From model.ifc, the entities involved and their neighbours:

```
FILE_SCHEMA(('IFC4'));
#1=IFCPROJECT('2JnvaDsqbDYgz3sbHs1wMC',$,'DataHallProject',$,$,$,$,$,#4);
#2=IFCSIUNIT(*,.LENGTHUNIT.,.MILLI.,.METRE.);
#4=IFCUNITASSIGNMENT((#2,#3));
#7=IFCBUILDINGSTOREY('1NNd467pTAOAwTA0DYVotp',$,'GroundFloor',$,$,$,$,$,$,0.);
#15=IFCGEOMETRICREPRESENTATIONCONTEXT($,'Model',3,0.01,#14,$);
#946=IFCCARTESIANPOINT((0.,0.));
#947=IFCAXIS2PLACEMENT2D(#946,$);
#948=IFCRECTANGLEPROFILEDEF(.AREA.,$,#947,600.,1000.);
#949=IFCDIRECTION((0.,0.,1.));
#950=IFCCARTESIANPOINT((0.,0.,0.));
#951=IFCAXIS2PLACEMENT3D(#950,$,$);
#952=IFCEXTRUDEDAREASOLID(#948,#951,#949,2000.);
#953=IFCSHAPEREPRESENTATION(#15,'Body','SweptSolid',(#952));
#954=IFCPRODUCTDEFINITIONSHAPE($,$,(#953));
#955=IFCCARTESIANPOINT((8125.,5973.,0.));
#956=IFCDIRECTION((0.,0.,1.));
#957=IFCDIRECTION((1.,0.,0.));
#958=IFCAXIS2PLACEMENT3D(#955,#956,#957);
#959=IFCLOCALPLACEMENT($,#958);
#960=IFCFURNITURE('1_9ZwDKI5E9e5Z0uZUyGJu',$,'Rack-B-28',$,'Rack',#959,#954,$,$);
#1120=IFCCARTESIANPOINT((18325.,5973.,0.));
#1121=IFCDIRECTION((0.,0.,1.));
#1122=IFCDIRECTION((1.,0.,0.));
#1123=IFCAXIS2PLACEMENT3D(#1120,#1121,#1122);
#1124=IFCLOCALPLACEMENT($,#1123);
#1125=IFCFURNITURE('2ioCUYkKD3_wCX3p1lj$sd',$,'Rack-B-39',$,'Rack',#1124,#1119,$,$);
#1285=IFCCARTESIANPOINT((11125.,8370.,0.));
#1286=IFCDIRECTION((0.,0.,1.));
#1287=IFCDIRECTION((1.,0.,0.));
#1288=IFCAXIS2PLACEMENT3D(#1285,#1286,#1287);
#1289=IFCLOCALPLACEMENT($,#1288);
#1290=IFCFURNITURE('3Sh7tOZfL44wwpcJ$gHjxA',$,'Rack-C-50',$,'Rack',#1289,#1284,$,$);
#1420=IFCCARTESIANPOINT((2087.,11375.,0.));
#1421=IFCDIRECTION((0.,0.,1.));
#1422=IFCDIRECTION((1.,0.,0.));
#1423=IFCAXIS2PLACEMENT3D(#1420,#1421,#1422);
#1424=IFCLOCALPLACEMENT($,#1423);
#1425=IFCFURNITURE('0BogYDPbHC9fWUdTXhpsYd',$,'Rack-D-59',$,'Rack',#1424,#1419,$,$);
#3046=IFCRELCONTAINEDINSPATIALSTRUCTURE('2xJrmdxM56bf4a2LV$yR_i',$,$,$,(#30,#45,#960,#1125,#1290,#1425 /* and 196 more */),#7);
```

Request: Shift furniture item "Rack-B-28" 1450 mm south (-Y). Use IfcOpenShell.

```python
import ifcopenshell
import ifcopenshell.api.geometry
import ifcopenshell.util.placement

model = ifcopenshell.open("model.ifc")

item = model.by_id(960)
matrix = ifcopenshell.util.placement.get_local_placement(item.ObjectPlacement)
matrix[1, 3] -= 1450.0
ifcopenshell.api.geometry.edit_object_placement(model, product=item, matrix=matrix, is_si=False)

print(ifcopenshell.util.placement.get_local_placement(item.ObjectPlacement).round(3) + 0.0)

model.write("model_updated.ifc")
```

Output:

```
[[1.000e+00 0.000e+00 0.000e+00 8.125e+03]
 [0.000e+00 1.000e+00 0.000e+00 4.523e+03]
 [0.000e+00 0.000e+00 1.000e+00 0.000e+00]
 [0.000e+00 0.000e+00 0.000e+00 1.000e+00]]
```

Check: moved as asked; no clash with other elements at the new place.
